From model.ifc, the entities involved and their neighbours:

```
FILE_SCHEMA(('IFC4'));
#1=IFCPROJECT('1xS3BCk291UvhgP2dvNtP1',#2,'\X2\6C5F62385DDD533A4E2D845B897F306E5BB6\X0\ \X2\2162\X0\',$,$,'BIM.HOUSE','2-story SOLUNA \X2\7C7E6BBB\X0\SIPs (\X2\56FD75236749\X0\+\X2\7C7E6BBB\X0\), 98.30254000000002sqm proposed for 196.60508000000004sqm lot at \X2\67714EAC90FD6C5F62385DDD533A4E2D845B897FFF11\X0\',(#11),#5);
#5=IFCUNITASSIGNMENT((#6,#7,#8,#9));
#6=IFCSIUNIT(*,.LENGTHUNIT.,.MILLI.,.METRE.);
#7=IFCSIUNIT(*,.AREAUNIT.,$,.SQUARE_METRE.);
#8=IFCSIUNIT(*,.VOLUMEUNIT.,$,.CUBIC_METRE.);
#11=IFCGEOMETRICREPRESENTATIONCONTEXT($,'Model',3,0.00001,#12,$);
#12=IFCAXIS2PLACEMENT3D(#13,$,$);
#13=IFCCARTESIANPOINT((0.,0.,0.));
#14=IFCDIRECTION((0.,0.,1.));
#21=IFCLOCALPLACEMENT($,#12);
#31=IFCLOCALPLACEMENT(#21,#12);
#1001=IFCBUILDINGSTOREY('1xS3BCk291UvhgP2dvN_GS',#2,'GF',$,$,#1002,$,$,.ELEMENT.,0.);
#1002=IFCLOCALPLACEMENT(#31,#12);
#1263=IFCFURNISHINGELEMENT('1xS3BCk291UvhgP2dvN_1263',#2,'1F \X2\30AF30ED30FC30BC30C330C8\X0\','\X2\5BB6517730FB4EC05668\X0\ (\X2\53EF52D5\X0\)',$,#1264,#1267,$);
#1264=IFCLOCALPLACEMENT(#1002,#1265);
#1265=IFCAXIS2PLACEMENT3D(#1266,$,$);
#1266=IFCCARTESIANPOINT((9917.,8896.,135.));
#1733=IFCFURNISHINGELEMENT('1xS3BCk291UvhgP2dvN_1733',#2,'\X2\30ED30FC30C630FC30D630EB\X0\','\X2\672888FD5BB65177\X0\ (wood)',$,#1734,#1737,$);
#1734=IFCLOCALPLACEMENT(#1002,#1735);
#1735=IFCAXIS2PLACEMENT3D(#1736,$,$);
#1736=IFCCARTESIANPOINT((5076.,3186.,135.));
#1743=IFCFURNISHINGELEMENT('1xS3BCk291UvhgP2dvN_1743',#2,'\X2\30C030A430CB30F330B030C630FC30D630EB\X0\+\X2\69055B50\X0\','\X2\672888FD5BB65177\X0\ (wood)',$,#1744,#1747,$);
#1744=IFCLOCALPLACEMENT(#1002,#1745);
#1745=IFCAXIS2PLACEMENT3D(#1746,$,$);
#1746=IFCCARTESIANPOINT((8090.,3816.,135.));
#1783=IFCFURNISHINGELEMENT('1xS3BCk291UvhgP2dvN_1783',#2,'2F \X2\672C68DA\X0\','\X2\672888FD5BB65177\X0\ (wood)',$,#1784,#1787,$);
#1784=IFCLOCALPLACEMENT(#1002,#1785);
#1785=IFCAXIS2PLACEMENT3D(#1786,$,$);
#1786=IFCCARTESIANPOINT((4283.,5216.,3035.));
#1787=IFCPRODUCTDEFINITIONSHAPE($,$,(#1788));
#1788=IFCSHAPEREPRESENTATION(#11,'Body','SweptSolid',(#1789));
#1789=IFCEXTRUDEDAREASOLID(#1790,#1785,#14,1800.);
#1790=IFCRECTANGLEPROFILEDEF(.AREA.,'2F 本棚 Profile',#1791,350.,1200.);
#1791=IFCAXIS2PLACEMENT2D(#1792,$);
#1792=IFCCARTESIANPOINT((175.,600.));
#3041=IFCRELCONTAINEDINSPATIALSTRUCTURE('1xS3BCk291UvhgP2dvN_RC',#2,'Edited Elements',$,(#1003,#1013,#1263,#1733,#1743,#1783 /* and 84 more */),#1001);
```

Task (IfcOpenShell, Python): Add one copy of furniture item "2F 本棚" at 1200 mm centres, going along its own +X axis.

```python
import ifcopenshell
import ifcopenshell.api.geometry
import ifcopenshell.api.root
import ifcopenshell.util.element
import ifcopenshell.util.placement
import ifcopenshell.util.unit

model = ifcopenshell.open("model.ifc")
unit_scale = ifcopenshell.util.unit.calculate_unit_scale(model)


def reuse_history(source, copy):
    """copy_class also copies each property set's owner history, people and application; keep the originals."""
    for rel in copy.IsDefinedBy:
        if rel.is_a("IfcRelDefinesByProperties") and (history := rel.RelatingPropertyDefinition.OwnerHistory):
            rel.RelatingPropertyDefinition.OwnerHistory = source.OwnerHistory
            ifcopenshell.util.element.remove_deep2(model, history)


source = model.by_guid("1xS3BCk291UvhgP2dvN_1783")
base = ifcopenshell.util.placement.get_local_placement(source.ObjectPlacement)
step = base[:3, 0] * 1.2 / unit_scale

for i in range(1, 2):
    copy = ifcopenshell.api.root.copy_class(model, product=source)
    copy.Representation = ifcopenshell.util.element.copy_deep(
        model, source.Representation, exclude=["IfcGeometricRepresentationContext", "IfcRepresentationMap"]
    )
    reuse_history(source, copy)
    matrix = base.copy()
    matrix[:3, 3] += i * step
    print("added at", matrix[:3, 3].round(3) + 0.0)
    ifcopenshell.api.geometry.edit_object_placement(model, product=copy, matrix=matrix, is_si=False)

model.write("model_updated.ifc")
```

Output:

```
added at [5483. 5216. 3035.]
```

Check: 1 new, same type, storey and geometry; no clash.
